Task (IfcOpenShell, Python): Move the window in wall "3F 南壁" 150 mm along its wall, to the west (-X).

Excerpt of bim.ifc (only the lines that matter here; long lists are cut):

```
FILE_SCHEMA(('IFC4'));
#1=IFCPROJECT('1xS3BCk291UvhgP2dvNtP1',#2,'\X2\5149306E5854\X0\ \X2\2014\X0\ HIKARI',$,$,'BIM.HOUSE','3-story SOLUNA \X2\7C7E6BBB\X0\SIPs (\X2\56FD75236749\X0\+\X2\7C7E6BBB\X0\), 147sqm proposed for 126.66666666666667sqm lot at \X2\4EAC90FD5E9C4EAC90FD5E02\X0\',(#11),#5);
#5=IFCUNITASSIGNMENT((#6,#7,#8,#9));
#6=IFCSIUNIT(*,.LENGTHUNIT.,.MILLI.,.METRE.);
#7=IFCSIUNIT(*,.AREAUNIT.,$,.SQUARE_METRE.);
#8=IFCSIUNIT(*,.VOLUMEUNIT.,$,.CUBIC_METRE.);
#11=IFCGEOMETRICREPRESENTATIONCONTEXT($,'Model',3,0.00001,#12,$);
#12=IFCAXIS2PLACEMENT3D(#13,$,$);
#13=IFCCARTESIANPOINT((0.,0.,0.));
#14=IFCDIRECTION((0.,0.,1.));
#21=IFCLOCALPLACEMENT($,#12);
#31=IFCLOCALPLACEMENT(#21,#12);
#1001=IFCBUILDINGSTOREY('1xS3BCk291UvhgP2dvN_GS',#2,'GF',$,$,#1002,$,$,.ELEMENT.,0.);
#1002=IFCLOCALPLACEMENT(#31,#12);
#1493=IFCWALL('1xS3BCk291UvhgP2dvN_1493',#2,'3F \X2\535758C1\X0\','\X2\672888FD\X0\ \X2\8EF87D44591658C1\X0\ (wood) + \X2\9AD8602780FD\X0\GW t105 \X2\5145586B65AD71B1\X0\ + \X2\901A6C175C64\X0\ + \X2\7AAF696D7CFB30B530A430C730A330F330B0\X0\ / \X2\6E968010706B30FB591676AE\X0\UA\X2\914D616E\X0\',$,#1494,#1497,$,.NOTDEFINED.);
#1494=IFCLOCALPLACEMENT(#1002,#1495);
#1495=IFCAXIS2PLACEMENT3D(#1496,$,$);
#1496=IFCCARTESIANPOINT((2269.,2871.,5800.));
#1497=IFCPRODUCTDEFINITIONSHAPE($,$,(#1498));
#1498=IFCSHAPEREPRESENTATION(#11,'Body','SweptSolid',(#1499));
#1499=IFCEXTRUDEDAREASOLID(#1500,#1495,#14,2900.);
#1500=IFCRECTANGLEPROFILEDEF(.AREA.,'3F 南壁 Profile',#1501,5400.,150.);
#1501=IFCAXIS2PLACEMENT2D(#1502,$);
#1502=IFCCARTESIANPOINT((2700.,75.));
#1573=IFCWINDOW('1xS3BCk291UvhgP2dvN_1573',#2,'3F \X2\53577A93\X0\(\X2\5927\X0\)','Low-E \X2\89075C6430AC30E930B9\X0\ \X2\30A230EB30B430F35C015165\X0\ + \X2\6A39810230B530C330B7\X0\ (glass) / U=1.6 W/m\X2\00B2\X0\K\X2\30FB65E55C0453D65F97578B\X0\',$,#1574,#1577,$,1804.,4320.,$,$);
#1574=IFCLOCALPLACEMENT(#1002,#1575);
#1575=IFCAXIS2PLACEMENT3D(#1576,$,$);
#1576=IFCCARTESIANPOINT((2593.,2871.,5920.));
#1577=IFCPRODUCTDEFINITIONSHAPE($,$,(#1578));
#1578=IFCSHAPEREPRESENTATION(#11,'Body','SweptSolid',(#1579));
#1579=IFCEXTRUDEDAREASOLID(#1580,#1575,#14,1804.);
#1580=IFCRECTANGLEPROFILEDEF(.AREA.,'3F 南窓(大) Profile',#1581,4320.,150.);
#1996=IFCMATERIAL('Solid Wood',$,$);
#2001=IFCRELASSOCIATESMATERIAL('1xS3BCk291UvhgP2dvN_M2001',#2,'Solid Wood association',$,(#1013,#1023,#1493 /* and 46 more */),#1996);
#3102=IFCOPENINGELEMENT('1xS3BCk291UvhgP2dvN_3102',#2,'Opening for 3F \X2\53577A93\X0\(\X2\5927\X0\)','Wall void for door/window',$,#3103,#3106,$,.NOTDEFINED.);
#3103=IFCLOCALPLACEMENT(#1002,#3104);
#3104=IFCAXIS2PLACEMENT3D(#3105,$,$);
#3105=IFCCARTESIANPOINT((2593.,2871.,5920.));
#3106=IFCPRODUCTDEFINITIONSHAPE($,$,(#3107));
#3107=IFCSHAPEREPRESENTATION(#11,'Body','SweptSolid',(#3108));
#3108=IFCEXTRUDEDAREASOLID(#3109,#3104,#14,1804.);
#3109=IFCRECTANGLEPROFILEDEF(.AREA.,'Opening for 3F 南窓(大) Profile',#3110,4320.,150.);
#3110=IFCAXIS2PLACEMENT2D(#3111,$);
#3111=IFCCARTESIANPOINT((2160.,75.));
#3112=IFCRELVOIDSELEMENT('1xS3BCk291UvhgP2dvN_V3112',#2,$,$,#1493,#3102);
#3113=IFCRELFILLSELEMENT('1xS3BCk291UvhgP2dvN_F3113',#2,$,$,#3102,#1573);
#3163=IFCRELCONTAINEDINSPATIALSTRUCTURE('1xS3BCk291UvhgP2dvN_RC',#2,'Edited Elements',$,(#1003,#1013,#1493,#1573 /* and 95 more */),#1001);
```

```python
import ifcopenshell
import ifcopenshell.api.geometry
import ifcopenshell.util.placement
import ifcopenshell.util.unit

model = ifcopenshell.open("bim.ifc")
unit_scale = ifcopenshell.util.unit.calculate_unit_scale(model)

window = model.by_id(1573)
opening = window.FillsVoids[0].RelatingOpeningElement
wall = opening.VoidsElements[0].RelatingBuildingElement

wall_matrix = ifcopenshell.util.placement.get_local_placement(wall.ObjectPlacement)
shift = wall_matrix[:3, 0] * -0.15 / unit_scale
before = ifcopenshell.util.placement.get_local_placement(window.ObjectPlacement)[:3, 3].copy()

# The window is not placed relative to its opening, so move both.
for product in (opening, window):
    matrix = ifcopenshell.util.placement.get_local_placement(product.ObjectPlacement)
    matrix[:3, 3] += shift
    ifcopenshell.api.geometry.edit_object_placement(model, product=product, matrix=matrix, is_si=False)

after = ifcopenshell.util.placement.get_local_placement(window.ObjectPlacement)[:3, 3]
print("window moved by", (after - before).round(3) + 0.0)

model.write("bim_edited.ifc")
```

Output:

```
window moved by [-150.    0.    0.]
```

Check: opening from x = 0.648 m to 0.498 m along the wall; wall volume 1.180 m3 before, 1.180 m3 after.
